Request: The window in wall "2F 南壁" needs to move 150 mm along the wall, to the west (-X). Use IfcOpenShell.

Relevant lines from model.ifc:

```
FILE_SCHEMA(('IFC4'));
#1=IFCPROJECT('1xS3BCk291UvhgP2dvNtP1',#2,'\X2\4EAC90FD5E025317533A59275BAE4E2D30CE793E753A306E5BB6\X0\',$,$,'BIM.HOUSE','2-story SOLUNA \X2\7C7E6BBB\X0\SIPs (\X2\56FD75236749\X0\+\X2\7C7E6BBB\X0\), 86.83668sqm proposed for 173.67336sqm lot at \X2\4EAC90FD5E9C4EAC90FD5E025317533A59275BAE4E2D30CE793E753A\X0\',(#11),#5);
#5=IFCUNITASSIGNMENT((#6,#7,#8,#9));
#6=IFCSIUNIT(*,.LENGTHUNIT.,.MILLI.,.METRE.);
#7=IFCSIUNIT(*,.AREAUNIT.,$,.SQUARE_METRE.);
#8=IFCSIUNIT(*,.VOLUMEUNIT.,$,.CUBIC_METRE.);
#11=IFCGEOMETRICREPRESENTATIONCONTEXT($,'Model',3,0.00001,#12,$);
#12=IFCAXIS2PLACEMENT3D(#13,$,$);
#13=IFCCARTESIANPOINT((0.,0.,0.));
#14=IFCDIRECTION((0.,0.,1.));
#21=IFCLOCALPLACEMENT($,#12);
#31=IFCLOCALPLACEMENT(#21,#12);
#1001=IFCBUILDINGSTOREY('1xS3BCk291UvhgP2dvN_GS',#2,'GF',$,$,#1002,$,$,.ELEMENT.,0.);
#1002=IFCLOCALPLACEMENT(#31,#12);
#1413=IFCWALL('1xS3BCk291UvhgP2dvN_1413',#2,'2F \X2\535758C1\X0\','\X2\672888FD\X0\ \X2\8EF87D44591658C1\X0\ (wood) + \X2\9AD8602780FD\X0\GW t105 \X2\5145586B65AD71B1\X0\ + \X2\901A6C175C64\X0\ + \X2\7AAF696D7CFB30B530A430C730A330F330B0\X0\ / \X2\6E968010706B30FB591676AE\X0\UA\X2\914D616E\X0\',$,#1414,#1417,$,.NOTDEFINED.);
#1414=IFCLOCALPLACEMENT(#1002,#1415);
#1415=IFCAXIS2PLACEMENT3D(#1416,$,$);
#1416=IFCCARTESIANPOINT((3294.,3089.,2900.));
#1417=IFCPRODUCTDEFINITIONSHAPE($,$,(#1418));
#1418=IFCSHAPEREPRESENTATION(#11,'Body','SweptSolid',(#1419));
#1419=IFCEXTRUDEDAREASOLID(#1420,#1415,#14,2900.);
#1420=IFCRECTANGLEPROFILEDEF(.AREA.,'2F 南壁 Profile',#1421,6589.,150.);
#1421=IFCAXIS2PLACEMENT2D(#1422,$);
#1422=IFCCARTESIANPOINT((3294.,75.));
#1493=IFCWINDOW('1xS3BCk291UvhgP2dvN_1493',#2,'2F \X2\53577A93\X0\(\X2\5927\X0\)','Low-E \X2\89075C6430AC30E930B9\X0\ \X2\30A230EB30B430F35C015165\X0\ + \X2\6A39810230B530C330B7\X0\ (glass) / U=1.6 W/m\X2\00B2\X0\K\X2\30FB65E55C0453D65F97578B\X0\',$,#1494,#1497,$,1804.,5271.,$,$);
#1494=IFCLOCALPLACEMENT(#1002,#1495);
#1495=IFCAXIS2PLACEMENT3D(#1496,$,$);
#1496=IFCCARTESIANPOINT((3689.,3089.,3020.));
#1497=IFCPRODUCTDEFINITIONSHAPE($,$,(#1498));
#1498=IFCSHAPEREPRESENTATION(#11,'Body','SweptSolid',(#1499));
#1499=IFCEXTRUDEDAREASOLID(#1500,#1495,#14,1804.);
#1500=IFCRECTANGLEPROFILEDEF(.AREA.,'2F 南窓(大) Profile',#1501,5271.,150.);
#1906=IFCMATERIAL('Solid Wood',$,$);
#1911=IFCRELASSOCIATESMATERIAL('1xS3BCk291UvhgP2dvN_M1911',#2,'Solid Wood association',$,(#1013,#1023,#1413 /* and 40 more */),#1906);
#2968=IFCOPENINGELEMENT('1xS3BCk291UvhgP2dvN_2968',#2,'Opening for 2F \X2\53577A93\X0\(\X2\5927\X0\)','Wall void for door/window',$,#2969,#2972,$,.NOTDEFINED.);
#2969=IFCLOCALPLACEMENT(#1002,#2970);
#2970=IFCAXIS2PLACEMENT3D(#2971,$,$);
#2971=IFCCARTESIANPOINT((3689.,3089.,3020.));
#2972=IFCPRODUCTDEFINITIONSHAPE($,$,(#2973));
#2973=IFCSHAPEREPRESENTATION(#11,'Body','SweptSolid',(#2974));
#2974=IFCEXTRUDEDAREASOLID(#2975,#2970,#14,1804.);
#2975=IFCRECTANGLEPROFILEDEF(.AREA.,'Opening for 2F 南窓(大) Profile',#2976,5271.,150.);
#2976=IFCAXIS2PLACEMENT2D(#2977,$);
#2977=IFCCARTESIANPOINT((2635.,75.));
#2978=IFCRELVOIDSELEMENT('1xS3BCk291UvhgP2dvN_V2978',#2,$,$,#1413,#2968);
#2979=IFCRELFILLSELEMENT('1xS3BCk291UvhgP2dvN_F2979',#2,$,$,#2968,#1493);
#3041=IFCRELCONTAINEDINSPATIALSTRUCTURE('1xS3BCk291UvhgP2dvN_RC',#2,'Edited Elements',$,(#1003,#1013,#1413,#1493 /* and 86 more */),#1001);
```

```python
import ifcopenshell
import ifcopenshell.api.geometry
import ifcopenshell.util.placement
import ifcopenshell.util.unit

model = ifcopenshell.open("model.ifc")
unit_scale = ifcopenshell.util.unit.calculate_unit_scale(model)

window = model.by_guid("1xS3BCk291UvhgP2dvN_1493")
opening = window.FillsVoids[0].RelatingOpeningElement
wall = opening.VoidsElements[0].RelatingBuildingElement

wall_matrix = ifcopenshell.util.placement.get_local_placement(wall.ObjectPlacement)
shift = wall_matrix[:3, 0] * -0.15 / unit_scale
before = ifcopenshell.util.placement.get_local_placement(window.ObjectPlacement)[:3, 3].copy()

# The window is not placed relative to its opening, so move both.
for product in (opening, window):
    matrix = ifcopenshell.util.placement.get_local_placement(product.ObjectPlacement)
    matrix[:3, 3] += shift
    ifcopenshell.api.geometry.edit_object_placement(model, product=product, matrix=matrix, is_si=False)

after = ifcopenshell.util.placement.get_local_placement(window.ObjectPlacement)[:3, 3]
print("window moved by", (after - before).round(3) + 0.0)

model.write("model_updated.ifc")
```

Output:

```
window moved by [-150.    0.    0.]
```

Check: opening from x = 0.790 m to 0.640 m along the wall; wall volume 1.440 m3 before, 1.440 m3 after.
